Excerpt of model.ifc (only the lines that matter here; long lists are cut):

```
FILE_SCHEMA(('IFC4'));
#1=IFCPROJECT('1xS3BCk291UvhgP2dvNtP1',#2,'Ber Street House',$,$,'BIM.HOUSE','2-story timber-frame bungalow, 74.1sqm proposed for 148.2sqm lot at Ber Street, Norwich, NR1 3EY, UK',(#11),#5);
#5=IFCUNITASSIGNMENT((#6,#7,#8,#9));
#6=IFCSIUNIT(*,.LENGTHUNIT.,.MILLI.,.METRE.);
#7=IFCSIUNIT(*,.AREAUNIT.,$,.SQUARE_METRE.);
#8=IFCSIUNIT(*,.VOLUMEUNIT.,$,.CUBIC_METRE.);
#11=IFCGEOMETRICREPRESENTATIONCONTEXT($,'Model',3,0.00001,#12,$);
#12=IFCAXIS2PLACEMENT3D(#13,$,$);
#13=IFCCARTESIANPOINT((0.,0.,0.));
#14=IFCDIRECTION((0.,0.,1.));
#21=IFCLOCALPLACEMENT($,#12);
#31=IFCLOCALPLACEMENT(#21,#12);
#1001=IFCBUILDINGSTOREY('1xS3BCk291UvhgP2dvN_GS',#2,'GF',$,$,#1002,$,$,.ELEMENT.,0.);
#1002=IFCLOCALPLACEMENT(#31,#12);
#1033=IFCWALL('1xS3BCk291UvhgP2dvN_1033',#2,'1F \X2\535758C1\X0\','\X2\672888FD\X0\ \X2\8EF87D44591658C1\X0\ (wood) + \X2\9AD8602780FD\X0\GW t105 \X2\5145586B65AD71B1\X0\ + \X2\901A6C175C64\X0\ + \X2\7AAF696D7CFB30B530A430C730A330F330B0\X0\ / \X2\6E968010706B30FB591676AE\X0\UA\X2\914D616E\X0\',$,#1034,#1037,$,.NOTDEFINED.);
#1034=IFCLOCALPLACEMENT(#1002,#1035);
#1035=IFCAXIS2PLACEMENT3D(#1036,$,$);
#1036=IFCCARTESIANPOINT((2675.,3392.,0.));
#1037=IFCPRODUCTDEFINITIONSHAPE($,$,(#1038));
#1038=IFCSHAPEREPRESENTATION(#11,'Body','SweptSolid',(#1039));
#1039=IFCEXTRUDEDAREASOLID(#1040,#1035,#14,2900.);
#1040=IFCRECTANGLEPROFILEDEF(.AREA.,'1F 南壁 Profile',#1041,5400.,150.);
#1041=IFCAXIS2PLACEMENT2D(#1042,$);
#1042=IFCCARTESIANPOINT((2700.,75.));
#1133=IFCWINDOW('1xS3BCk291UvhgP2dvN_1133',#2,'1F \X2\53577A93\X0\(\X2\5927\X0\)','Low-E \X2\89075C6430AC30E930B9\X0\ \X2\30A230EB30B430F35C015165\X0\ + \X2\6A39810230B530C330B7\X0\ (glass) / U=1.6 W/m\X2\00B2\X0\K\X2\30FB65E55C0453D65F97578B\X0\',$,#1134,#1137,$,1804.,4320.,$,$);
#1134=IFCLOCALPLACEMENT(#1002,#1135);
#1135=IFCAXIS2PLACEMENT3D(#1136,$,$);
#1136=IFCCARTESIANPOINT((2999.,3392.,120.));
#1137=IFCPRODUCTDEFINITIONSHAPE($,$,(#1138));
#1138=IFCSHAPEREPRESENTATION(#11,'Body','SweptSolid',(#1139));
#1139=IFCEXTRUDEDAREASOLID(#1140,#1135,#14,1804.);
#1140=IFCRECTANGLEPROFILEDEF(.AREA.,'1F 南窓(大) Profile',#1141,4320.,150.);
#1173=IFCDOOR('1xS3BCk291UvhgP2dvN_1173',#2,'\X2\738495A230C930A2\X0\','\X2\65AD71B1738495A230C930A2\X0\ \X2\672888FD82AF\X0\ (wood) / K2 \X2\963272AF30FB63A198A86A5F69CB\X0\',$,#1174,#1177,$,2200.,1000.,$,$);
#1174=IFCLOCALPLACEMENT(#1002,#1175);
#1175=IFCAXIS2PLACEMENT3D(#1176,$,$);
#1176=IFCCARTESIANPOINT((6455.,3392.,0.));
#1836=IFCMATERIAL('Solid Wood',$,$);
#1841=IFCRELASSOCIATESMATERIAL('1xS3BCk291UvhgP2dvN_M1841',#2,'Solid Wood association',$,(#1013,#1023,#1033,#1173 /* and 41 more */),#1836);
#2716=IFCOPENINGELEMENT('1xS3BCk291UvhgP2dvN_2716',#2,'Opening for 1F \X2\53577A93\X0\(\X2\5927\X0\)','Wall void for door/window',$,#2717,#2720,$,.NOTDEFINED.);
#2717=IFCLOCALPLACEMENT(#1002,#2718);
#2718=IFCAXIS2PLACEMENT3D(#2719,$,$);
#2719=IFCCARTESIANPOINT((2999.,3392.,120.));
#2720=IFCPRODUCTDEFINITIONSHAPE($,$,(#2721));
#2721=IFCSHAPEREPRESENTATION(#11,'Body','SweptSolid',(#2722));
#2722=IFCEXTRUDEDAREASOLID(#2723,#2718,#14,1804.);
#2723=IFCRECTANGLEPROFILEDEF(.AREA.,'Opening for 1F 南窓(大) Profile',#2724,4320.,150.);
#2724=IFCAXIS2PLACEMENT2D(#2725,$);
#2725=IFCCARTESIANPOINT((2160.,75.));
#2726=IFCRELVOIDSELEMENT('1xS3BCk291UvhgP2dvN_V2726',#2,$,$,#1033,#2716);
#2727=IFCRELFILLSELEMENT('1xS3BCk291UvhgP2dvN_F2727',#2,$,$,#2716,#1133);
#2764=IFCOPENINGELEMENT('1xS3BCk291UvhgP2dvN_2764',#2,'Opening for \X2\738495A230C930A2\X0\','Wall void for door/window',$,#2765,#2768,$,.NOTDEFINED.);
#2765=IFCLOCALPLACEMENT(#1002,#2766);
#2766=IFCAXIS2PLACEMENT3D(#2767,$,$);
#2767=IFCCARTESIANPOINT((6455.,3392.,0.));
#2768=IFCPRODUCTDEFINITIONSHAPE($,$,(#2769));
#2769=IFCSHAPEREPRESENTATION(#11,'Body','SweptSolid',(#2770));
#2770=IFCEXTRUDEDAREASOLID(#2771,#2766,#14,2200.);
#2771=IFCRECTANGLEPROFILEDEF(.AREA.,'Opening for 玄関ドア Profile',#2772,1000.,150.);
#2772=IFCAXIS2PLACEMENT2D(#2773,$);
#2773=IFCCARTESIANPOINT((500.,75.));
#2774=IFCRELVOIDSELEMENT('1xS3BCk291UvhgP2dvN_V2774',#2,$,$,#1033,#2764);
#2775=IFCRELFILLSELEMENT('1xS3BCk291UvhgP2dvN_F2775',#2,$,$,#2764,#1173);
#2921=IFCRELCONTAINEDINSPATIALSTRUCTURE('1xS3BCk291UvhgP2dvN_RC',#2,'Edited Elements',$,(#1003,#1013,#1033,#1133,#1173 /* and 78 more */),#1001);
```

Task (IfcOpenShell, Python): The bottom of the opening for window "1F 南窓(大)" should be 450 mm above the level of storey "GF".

```python
import numpy as np
import ifcopenshell
import ifcopenshell.api.geometry
import ifcopenshell.geom
import ifcopenshell.util.element
import ifcopenshell.util.placement
import ifcopenshell.util.shape
import ifcopenshell.util.unit

model = ifcopenshell.open("model.ifc")
unit_scale = ifcopenshell.util.unit.calculate_unit_scale(model)

window = model.by_guid("1xS3BCk291UvhgP2dvN_1133")
opening = window.FillsVoids[0].RelatingOpeningElement
storey = ifcopenshell.util.element.get_container(window, ifc_class="IfcBuildingStorey")
level = ifcopenshell.util.placement.get_local_placement(storey.ObjectPlacement)[2, 3]

# The opening's origin need not be at the sill, so measure its lowest point.
shape = ifcopenshell.geom.create_shape(ifcopenshell.geom.settings(), opening)
bottom = ifcopenshell.util.shape.get_shape_bottom_elevation(shape, shape.geometry) / unit_scale
dz = level + 0.45 / unit_scale - bottom

shift = np.array([0.0, 0.0, dz])
# The window is not placed relative to its opening, so move both.
for product in (opening, window):
    matrix = ifcopenshell.util.placement.get_local_placement(product.ObjectPlacement)
    matrix[:3, 3] += shift
    ifcopenshell.api.geometry.edit_object_placement(model, product=product, matrix=matrix, is_si=False)

print(f"moved by {dz * unit_scale:+.3f} m")

model.write("model_rev.ifc")
```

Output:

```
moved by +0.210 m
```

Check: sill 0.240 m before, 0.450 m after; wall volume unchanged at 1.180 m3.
